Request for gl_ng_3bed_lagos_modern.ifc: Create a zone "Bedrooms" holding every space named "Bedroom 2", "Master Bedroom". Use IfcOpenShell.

First a look at what the model holds.

```python
import ifcopenshell

model = ifcopenshell.open("gl_ng_3bed_lagos_modern.ifc")
print(model.schema)
seen = {}
for space in model.by_type("IfcSpace"):
    seen[space.LongName] = seen.get(space.LongName, 0) + 1
for name, count in sorted(seen.items(), key=str):
    print(count, "x", name)
print("zones:", [z.Name for z in model.by_type("IfcZone")][:20])
```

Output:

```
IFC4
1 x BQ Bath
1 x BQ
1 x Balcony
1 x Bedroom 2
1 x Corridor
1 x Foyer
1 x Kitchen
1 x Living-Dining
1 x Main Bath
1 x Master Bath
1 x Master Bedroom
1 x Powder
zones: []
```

```python
import ifcopenshell
import ifcopenshell.api.group
import ifcopenshell.api.root

model = ifcopenshell.open("gl_ng_3bed_lagos_modern.ifc")

names = {"Bedroom 2", "Master Bedroom"}
spaces = [s for s in model.by_type("IfcSpace") if s.LongName in names]

zone = ifcopenshell.api.root.create_entity(model, ifc_class="IfcZone", name="Bedrooms")
ifcopenshell.api.group.assign_group(model, products=spaces, group=zone)
print(len(spaces), "spaces in", zone.Name)

model.write("gl_ng_3bed_lagos_modern_rev.ifc")
```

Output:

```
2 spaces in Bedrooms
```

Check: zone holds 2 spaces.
